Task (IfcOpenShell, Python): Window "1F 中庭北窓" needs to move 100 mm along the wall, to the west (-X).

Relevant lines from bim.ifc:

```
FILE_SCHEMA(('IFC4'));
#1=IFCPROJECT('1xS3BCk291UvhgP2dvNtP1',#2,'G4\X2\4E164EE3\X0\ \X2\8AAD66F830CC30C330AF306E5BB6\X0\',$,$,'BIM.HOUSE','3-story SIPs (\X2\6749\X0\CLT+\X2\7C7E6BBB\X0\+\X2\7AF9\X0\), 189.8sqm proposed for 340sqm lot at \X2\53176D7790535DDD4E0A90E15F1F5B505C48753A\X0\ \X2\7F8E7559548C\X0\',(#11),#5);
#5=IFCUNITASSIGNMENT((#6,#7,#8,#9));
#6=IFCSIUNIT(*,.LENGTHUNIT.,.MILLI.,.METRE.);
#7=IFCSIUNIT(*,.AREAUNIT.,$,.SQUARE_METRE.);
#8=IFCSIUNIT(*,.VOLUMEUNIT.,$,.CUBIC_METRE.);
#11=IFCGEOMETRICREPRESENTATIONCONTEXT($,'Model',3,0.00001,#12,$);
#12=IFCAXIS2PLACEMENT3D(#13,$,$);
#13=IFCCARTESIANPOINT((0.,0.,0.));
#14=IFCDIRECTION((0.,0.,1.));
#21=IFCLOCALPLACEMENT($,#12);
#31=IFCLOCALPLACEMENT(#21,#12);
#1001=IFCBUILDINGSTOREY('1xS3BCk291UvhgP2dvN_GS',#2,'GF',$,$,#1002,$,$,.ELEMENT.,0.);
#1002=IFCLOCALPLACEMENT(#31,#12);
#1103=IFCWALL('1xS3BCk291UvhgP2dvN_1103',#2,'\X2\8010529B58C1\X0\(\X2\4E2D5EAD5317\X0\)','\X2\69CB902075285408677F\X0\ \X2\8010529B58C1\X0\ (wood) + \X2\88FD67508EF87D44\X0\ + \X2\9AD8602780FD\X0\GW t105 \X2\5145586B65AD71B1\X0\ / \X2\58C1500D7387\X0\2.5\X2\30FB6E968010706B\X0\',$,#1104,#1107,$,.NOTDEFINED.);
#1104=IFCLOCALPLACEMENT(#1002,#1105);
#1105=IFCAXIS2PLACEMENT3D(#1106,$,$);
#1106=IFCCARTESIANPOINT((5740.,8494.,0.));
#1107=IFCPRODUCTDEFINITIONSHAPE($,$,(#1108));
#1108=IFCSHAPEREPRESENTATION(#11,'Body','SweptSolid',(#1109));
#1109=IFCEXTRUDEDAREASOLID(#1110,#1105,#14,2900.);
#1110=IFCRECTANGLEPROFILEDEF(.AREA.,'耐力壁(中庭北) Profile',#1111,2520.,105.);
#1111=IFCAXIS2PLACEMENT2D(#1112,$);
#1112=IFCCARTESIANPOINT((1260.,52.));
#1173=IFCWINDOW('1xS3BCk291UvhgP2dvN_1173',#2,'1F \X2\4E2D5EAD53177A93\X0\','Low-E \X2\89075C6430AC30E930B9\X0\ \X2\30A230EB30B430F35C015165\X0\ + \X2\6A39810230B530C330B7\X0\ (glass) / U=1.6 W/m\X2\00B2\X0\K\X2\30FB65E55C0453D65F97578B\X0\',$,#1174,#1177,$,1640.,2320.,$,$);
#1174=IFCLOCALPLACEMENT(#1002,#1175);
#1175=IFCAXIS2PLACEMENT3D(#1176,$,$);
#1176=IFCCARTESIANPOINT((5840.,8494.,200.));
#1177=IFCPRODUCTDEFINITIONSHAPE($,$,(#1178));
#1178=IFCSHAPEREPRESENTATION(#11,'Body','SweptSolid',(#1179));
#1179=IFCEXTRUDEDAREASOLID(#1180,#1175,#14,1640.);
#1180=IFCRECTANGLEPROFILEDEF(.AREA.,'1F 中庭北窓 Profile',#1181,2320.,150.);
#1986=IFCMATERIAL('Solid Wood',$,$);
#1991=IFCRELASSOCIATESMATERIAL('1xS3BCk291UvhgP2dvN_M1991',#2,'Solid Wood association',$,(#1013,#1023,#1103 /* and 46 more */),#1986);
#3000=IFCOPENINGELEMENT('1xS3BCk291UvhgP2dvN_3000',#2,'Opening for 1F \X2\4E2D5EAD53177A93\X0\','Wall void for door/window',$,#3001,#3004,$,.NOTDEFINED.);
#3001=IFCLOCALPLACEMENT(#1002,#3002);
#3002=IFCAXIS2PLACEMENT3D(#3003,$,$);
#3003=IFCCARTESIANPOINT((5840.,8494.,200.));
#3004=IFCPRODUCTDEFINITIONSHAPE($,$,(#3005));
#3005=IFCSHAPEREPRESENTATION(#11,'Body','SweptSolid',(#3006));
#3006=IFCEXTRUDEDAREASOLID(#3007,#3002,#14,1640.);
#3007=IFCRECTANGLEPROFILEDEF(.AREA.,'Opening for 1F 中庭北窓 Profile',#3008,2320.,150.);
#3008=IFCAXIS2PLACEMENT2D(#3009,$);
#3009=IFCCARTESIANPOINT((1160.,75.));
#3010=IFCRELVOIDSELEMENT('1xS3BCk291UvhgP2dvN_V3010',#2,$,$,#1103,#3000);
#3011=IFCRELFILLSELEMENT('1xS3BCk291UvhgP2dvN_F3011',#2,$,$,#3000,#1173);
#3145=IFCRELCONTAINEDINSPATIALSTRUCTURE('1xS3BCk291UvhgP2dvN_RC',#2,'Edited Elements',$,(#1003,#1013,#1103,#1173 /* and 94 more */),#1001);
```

```python
import ifcopenshell
import ifcopenshell.api.geometry
import ifcopenshell.util.placement

model = ifcopenshell.open("bim.ifc")

window = model.by_guid("1xS3BCk291UvhgP2dvN_1173")
opening = window.FillsVoids[0].RelatingOpeningElement
wall = opening.VoidsElements[0].RelatingBuildingElement

wall_matrix = ifcopenshell.util.placement.get_local_placement(wall.ObjectPlacement)
shift = wall_matrix[:3, 0] * -100.0
before = ifcopenshell.util.placement.get_local_placement(window.ObjectPlacement)[:3, 3].copy()

# The window is not placed relative to its opening, so move both.
for product in (opening, window):
    matrix = ifcopenshell.util.placement.get_local_placement(product.ObjectPlacement)
    matrix[:3, 3] += shift
    ifcopenshell.api.geometry.edit_object_placement(model, product=product, matrix=matrix, is_si=False)

after = ifcopenshell.util.placement.get_local_placement(window.ObjectPlacement)[:3, 3]
print("window moved by", (after - before).round(3) + 0.0)

model.write("bim_rev.ifc")
```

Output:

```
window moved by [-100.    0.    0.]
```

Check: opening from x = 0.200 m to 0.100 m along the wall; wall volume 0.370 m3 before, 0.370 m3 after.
